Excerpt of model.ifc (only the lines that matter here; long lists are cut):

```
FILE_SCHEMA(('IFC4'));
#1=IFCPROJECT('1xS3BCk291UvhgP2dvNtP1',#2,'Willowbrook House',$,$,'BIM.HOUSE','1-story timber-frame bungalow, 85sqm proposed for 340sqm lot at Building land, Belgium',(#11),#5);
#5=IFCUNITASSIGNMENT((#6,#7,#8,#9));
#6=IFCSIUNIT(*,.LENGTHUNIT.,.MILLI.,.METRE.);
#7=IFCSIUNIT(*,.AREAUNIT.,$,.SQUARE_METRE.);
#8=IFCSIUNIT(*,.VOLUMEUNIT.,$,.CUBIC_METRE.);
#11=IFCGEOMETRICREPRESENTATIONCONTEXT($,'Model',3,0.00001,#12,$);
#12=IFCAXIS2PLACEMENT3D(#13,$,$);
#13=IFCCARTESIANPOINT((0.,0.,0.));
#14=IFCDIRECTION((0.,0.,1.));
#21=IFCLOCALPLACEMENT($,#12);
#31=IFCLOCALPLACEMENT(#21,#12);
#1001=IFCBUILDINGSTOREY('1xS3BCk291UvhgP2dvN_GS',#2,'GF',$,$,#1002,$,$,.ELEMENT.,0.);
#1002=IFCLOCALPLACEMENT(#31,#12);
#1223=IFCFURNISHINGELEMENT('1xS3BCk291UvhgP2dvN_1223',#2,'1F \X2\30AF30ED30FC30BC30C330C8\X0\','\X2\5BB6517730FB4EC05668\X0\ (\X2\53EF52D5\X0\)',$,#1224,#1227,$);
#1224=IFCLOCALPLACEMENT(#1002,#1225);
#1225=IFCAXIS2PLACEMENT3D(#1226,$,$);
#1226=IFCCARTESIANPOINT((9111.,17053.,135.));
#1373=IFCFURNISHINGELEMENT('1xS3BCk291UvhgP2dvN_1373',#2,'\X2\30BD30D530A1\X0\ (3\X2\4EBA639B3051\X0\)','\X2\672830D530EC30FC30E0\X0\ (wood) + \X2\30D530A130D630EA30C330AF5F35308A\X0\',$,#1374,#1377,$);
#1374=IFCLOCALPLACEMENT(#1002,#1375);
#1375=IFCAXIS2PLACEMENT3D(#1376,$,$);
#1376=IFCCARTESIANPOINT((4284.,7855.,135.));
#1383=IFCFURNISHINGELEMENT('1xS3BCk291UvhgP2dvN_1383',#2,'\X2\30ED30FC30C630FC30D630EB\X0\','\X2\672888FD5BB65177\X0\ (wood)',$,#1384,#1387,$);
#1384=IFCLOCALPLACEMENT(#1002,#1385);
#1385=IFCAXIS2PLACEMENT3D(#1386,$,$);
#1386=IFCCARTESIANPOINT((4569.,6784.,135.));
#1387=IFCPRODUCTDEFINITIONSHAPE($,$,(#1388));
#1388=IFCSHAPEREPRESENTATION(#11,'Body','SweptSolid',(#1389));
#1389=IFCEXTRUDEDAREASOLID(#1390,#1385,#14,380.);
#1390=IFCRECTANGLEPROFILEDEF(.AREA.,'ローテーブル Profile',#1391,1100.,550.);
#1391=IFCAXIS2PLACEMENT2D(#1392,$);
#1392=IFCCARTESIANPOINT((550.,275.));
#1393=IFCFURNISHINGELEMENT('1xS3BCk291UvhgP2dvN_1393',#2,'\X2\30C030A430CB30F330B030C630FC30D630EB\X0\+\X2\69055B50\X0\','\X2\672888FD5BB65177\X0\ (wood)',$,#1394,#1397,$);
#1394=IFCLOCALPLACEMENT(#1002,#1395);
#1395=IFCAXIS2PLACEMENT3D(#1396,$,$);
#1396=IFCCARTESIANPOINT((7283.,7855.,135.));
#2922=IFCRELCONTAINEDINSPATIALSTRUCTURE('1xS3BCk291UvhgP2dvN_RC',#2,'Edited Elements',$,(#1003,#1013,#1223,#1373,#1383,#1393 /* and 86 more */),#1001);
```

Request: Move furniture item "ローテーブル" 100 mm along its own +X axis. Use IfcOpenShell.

```python
import ifcopenshell
import ifcopenshell.api.geometry
import ifcopenshell.util.placement
import ifcopenshell.util.unit

model = ifcopenshell.open("model.ifc")
unit_scale = ifcopenshell.util.unit.calculate_unit_scale(model)

item = model.by_id(1383)
matrix = ifcopenshell.util.placement.get_local_placement(item.ObjectPlacement)
matrix[:3, 3] += matrix[:3, 0] * 0.1 / unit_scale
ifcopenshell.api.geometry.edit_object_placement(model, product=item, matrix=matrix, is_si=False)

print(ifcopenshell.util.placement.get_local_placement(item.ObjectPlacement).round(3) + 0.0)

model.write("model_rev.ifc")
```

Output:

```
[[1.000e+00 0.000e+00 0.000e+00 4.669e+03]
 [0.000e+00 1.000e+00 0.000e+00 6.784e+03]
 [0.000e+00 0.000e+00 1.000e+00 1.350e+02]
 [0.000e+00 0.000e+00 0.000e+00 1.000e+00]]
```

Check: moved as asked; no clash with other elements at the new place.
